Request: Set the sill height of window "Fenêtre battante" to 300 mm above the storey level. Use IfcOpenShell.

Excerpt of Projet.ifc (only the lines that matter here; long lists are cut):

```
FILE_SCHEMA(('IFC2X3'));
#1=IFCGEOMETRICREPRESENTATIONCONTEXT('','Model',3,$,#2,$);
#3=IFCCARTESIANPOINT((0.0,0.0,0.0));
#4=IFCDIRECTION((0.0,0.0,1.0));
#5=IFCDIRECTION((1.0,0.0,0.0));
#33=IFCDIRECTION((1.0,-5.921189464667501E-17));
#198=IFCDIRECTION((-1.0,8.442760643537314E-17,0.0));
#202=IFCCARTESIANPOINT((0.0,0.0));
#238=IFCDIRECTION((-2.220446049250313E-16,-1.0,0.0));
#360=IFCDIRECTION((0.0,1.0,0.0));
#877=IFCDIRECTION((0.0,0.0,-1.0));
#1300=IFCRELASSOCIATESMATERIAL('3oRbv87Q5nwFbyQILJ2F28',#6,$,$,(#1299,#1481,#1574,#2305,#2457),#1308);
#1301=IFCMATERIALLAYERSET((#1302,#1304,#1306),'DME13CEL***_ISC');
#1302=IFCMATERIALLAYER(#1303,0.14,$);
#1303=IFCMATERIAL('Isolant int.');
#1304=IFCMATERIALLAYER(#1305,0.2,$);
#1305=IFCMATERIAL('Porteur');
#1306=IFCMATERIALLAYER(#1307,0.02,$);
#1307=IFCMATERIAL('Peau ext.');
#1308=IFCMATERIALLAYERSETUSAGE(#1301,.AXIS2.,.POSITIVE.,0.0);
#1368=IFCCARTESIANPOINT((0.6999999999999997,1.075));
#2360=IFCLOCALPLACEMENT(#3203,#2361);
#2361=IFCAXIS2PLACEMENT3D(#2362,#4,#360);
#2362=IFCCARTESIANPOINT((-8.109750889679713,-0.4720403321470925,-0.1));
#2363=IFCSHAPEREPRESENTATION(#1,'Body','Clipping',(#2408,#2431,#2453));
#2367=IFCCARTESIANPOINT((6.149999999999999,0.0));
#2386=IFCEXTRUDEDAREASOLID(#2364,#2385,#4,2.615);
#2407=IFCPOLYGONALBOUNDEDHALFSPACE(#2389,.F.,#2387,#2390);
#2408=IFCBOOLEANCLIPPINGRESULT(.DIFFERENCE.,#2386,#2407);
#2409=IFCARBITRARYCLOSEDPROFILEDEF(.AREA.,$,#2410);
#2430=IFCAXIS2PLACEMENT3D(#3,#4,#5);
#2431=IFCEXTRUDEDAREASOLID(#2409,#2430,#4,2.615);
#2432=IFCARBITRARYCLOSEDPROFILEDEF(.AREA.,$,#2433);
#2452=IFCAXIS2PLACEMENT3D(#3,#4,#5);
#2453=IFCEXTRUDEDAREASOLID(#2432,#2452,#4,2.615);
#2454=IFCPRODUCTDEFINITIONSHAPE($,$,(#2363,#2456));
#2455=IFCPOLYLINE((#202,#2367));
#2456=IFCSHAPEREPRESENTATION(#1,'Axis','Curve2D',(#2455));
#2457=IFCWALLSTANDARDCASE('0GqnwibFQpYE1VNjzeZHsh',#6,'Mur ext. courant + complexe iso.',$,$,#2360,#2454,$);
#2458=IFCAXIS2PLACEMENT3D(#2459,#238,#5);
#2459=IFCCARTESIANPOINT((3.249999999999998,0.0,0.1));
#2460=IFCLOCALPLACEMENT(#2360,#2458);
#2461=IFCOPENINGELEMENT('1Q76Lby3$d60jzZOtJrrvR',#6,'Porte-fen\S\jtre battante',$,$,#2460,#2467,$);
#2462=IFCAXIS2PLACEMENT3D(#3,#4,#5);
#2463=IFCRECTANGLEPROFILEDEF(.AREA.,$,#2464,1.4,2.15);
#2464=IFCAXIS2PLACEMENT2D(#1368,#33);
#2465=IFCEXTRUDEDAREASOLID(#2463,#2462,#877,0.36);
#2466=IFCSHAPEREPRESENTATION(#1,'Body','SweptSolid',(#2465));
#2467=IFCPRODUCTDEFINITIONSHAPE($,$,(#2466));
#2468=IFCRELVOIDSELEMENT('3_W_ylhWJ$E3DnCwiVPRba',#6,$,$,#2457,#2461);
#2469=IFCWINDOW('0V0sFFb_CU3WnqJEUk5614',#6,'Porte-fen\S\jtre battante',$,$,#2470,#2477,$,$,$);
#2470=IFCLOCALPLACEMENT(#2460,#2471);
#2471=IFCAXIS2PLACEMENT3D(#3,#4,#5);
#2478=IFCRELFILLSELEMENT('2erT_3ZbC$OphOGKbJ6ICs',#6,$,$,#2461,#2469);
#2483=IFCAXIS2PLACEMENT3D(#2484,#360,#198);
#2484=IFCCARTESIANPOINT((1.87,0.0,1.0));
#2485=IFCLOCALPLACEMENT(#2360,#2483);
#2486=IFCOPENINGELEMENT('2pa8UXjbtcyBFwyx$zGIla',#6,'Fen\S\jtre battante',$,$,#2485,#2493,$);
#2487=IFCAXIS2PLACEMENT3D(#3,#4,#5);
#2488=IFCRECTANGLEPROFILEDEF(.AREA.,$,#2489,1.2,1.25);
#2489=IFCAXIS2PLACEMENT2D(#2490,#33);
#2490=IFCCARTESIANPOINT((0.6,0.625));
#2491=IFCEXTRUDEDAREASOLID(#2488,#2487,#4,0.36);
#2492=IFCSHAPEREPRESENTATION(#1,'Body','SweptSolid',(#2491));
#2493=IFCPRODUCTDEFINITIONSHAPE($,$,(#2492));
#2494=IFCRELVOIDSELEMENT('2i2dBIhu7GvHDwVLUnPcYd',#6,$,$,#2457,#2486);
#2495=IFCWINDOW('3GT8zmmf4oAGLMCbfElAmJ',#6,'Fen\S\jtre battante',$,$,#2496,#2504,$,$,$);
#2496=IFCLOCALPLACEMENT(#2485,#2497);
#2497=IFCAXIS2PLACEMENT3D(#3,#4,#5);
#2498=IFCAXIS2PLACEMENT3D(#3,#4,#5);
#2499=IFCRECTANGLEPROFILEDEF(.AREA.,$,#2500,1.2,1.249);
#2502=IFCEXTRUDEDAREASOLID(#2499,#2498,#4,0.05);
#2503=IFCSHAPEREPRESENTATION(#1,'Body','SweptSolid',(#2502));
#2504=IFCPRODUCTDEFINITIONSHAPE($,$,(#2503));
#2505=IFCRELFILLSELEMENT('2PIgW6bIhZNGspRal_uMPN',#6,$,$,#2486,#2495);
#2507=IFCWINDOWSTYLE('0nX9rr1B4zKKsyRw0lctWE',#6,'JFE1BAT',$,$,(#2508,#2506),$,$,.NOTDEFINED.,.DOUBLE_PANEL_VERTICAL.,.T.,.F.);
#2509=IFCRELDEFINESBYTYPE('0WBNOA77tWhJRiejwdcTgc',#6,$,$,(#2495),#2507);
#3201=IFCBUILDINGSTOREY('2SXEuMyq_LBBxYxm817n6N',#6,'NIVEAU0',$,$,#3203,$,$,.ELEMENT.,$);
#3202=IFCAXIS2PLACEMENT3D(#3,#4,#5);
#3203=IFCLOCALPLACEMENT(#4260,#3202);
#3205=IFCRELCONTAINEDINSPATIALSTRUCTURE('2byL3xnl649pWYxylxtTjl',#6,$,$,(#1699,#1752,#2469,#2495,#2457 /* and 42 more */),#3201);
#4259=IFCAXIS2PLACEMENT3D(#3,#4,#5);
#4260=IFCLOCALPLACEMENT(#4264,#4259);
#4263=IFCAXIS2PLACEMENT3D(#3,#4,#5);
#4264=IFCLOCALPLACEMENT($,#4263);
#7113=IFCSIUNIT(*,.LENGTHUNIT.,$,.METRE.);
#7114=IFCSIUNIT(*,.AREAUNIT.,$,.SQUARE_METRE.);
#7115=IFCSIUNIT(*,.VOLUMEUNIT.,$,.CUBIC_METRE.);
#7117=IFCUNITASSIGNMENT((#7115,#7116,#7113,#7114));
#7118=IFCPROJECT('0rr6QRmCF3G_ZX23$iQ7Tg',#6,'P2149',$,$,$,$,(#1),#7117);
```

```python
import numpy as np
import ifcopenshell
import ifcopenshell.api.geometry
import ifcopenshell.geom
import ifcopenshell.util.element
import ifcopenshell.util.placement
import ifcopenshell.util.shape
import ifcopenshell.util.unit

model = ifcopenshell.open("Projet.ifc")
unit_scale = ifcopenshell.util.unit.calculate_unit_scale(model)

window = model.by_guid("3GT8zmmf4oAGLMCbfElAmJ")
opening = window.FillsVoids[0].RelatingOpeningElement
storey = ifcopenshell.util.element.get_container(window, ifc_class="IfcBuildingStorey")
level = ifcopenshell.util.placement.get_local_placement(storey.ObjectPlacement)[2, 3]

# The opening's origin need not be at the sill, so measure its lowest point.
shape = ifcopenshell.geom.create_shape(ifcopenshell.geom.settings(), opening)
bottom = ifcopenshell.util.shape.get_shape_bottom_elevation(shape, shape.geometry) / unit_scale
dz = level + 0.3 / unit_scale - bottom

shift = np.array([0.0, 0.0, dz])
# The window is placed relative to its opening, so it follows when the opening moves.
matrix = ifcopenshell.util.placement.get_local_placement(opening.ObjectPlacement)
matrix[:3, 3] += shift
ifcopenshell.api.geometry.edit_object_placement(
    model, product=opening, matrix=matrix, is_si=False, should_transform_children=True
)

print(f"moved by {dz * unit_scale:+.3f} m")

model.write("Projet_v2.ifc")
```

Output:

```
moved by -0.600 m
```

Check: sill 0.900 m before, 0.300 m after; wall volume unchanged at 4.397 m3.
